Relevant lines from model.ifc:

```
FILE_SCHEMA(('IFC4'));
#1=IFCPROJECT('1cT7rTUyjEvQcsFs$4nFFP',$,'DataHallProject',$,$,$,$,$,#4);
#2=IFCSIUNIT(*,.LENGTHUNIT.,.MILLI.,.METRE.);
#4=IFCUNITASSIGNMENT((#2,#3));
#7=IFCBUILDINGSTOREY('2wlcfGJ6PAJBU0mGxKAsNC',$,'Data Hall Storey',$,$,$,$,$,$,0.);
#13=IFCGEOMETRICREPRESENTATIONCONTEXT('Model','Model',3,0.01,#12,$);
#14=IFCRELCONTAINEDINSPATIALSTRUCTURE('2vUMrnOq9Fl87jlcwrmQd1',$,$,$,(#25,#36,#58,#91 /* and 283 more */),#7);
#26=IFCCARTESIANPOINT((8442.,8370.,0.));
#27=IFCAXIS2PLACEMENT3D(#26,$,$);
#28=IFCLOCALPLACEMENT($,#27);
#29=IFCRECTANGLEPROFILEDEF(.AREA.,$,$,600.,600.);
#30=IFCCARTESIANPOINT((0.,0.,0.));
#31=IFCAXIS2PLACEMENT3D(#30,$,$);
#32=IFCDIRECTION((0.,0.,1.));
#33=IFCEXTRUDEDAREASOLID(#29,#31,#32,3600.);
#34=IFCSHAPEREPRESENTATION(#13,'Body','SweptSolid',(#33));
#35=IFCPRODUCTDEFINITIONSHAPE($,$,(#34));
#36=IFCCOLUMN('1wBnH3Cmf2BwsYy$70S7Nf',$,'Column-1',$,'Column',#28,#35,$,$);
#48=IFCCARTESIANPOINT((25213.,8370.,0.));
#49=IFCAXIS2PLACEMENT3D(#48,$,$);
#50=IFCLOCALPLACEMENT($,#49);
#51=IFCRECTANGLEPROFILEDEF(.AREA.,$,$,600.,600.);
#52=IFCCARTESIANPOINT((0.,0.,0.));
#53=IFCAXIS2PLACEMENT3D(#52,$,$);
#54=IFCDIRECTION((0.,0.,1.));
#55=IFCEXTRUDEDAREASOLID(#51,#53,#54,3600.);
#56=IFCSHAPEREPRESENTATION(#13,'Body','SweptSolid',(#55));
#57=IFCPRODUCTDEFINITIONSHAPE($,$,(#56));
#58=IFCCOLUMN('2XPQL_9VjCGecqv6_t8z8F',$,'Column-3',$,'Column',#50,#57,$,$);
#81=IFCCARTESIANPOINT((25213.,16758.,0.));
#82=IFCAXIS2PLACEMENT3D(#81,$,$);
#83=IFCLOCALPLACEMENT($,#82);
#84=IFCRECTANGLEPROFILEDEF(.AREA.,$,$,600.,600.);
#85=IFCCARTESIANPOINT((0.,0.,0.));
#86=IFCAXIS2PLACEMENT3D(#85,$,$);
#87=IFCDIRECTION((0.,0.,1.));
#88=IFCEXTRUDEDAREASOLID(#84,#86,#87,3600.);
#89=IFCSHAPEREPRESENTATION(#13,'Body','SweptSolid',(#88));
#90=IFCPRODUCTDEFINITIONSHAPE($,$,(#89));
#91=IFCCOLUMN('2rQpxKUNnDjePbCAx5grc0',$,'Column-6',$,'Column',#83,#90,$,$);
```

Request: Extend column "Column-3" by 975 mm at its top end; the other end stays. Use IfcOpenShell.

```python
import ifcopenshell

model = ifcopenshell.open("model.ifc")

member = model.by_id(58)
change = 975.0

# The extrusion runs towards the end named, so only its depth changes.
body = next(r for r in member.Representation.Representations if r.RepresentationIdentifier == "Body")
solid = body.Items[0]
old_length = solid.Depth
solid.Depth += change

print(f"length {old_length:g} -> {solid.Depth:g}")

model.write("model-out.ifc")
```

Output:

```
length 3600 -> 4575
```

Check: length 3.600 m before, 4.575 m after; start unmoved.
